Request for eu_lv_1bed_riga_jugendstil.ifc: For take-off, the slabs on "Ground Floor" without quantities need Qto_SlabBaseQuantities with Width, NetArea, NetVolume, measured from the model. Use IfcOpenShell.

First a look at what the model holds.

```python
import ifcopenshell
import ifcopenshell.util.element
import ifcopenshell.util.unit

model = ifcopenshell.open("eu_lv_1bed_riga_jugendstil.ifc")
print(model.schema)
for unit_type in ("LENGTHUNIT", "AREAUNIT", "VOLUMEUNIT"):
    print(unit_type, ifcopenshell.util.unit.calculate_unit_scale(model, unit_type))
storey = next(s for s in model.by_type("IfcBuildingStorey") if s.Name == "Ground Floor")
slabs = [e for e in ifcopenshell.util.element.get_decomposition(storey) if e.is_a("IfcSlab")]
for e in sorted(slabs, key=lambda e: e.id()):
    print(e.id(), e.is_a(), e.Name, list(ifcopenshell.util.element.get_psets(e, qtos_only=True)), sep=" | ")
```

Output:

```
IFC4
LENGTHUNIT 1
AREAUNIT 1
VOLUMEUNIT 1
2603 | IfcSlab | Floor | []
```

```python
import ifcopenshell
import ifcopenshell.api.pset
import ifcopenshell.geom
import ifcopenshell.util.element
import ifcopenshell.util.shape
import ifcopenshell.util.unit

model = ifcopenshell.open("eu_lv_1bed_riga_jugendstil.ifc")
unit_scale = ifcopenshell.util.unit.calculate_unit_scale(model)
area_scale = ifcopenshell.util.unit.calculate_unit_scale(model, "AREAUNIT")
volume_scale = ifcopenshell.util.unit.calculate_unit_scale(model, "VOLUMEUNIT")
settings = ifcopenshell.geom.settings()

storey = next(s for s in model.by_type("IfcBuildingStorey") if s.Name == "Ground Floor")
slabs = [e for e in ifcopenshell.util.element.get_decomposition(storey) if e.is_a("IfcSlab")]

for e in sorted(slabs, key=lambda e: e.id()):
    if ifcopenshell.util.element.get_psets(e, qtos_only=True, should_inherit=False):
        continue
    # Geometry comes back in metres, in the element's own axes.
    shape = ifcopenshell.geom.create_shape(settings, e)
    values = {
        "Width": ifcopenshell.util.shape.get_z(shape.geometry) / unit_scale,
        "NetArea": ifcopenshell.util.shape.get_footprint_area(shape.geometry) / area_scale,
        "NetVolume": ifcopenshell.util.shape.get_volume(shape.geometry) / volume_scale,
    }
    qto = ifcopenshell.api.pset.add_qto(model, product=e, name="Qto_SlabBaseQuantities")
    ifcopenshell.api.pset.edit_qto(model, qto=qto, properties=values)
    print(e.id(), {k: round(v, 3) for k, v in values.items()})

model.write("eu_lv_1bed_riga_jugendstil_edited.ifc")
```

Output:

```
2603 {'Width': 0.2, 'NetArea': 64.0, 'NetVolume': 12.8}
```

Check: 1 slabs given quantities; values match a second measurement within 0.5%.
